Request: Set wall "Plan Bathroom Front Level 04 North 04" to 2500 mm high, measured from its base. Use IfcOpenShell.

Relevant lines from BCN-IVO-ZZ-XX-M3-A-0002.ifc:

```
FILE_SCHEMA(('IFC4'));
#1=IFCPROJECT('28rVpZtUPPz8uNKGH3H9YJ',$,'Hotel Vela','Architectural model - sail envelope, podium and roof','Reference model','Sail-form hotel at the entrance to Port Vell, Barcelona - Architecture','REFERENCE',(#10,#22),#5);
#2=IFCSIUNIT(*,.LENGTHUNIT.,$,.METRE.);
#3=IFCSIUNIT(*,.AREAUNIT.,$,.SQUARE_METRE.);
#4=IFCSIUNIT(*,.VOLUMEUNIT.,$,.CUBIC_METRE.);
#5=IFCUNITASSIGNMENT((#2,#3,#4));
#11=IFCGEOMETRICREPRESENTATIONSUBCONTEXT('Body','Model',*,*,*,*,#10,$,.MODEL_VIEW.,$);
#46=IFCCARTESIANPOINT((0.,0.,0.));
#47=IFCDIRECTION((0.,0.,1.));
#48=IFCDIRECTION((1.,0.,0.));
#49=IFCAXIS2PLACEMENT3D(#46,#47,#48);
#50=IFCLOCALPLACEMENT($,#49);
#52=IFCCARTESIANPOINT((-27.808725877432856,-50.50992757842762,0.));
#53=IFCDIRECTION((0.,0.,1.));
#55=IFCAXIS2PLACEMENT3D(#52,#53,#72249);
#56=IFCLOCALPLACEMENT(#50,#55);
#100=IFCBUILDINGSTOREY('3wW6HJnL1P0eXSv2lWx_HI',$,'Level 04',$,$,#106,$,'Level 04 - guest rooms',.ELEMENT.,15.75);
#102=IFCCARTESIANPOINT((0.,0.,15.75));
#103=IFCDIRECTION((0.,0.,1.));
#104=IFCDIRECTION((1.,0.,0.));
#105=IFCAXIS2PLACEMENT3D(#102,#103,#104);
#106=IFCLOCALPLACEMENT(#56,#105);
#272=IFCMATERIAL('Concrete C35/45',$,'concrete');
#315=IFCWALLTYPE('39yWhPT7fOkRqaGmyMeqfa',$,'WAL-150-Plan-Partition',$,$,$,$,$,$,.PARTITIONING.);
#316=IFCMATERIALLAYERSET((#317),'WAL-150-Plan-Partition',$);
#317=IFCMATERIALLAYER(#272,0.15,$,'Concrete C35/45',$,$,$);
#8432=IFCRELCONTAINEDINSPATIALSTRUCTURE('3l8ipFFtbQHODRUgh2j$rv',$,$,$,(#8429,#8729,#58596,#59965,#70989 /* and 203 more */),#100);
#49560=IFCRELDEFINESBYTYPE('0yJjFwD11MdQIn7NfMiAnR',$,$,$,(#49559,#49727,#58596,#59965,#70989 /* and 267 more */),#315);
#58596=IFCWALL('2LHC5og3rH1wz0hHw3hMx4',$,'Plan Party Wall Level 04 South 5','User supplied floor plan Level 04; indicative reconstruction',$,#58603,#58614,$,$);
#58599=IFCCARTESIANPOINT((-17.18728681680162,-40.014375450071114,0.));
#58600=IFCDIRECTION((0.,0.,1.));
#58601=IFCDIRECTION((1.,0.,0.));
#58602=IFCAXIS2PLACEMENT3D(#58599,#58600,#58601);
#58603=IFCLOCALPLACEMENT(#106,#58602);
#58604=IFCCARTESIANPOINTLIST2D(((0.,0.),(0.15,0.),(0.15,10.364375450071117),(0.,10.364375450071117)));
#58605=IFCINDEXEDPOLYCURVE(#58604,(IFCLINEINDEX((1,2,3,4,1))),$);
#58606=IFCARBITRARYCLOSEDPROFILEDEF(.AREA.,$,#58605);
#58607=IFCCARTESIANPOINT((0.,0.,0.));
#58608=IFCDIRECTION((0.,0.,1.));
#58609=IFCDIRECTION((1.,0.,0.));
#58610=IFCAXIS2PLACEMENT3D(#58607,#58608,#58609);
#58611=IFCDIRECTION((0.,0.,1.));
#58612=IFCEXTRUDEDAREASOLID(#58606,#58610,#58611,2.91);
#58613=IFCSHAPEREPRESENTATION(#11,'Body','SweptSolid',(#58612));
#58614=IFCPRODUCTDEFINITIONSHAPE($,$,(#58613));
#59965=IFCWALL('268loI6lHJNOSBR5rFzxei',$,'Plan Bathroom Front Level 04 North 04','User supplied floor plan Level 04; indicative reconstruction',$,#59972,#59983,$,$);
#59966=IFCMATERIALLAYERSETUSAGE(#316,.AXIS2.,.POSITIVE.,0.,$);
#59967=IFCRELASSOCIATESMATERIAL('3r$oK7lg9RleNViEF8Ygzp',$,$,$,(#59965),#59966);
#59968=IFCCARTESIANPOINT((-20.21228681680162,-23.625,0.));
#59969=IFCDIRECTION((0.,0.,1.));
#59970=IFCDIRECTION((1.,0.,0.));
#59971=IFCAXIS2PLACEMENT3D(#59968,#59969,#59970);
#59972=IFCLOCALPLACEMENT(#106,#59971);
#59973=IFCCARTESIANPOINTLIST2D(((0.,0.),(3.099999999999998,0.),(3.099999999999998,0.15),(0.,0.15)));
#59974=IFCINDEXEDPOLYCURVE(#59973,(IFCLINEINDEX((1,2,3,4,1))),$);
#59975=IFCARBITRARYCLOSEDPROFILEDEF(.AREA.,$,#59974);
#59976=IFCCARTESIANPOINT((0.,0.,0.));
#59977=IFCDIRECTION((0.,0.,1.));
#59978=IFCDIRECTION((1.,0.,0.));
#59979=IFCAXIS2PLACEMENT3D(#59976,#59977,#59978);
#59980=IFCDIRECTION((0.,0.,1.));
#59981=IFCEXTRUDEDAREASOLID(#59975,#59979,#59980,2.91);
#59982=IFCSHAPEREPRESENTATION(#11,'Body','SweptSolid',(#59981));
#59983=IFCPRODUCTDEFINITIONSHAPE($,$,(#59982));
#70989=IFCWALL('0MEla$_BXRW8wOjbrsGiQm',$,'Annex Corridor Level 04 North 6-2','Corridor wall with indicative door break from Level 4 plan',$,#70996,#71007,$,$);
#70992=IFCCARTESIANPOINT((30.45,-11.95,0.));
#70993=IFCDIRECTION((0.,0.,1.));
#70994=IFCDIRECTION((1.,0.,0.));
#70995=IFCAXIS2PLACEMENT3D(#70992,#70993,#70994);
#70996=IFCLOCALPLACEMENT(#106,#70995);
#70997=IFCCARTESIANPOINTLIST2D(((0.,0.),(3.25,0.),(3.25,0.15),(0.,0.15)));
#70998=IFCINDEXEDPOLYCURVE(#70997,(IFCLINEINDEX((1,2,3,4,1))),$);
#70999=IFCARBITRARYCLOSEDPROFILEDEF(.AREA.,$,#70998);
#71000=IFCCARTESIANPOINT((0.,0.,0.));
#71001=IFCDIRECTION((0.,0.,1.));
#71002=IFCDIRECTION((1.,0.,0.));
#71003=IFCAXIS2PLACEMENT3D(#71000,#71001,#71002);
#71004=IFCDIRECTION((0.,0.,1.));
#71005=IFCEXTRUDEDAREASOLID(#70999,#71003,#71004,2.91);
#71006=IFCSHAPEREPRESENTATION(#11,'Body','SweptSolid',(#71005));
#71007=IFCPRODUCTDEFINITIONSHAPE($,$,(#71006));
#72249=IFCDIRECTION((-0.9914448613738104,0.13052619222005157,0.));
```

```python
import ifcopenshell
import ifcopenshell.geom
import ifcopenshell.util.representation
import ifcopenshell.util.shape

model = ifcopenshell.open("BCN-IVO-ZZ-XX-M3-A-0002.ifc")
settings = ifcopenshell.geom.settings()


def volume(element):
    """Net volume in cubic metres, openings subtracted."""
    shape = ifcopenshell.geom.create_shape(settings, element)
    return ifcopenshell.util.shape.get_volume(shape.geometry)


wall = model.by_id(59965)
before = volume(wall)

body = ifcopenshell.util.representation.get_representation(wall, "Model", "Body")
solid = body.Items[0]
old_height = solid.Depth
solid.Depth = 2.5
after = volume(wall)

print(f"height {old_height:g} -> {solid.Depth:g}, volume {before:.3f} -> {after:.3f} m3")

model.write("BCN-IVO-ZZ-XX-M3-A-0002-out.ifc")
```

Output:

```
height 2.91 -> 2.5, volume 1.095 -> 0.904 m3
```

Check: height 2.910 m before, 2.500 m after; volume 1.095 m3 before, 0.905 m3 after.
